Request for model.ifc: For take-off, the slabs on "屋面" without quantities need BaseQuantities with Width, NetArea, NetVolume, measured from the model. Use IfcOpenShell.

First a look at what the model holds.

```python
import ifcopenshell
import ifcopenshell.util.element
import ifcopenshell.util.unit

model = ifcopenshell.open("model.ifc")
print(model.schema)
for unit_type in ("LENGTHUNIT", "AREAUNIT", "VOLUMEUNIT"):
    print(unit_type, ifcopenshell.util.unit.calculate_unit_scale(model, unit_type))
storey = next(s for s in model.by_type("IfcBuildingStorey") if s.Name == "屋面")
slabs = [e for e in ifcopenshell.util.element.get_decomposition(storey) if e.is_a("IfcSlab")]
for e in sorted(slabs, key=lambda e: e.id()):
    print(e.id(), e.is_a(), e.Name, list(ifcopenshell.util.element.get_psets(e, qtos_only=True)), sep=" | ")
```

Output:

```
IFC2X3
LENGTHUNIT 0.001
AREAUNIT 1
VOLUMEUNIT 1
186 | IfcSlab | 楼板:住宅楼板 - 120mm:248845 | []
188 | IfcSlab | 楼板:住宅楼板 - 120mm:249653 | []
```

```python
import ifcopenshell
import ifcopenshell.api.pset
import ifcopenshell.geom
import ifcopenshell.util.element
import ifcopenshell.util.shape
import ifcopenshell.util.unit

model = ifcopenshell.open("model.ifc")
unit_scale = ifcopenshell.util.unit.calculate_unit_scale(model)
area_scale = ifcopenshell.util.unit.calculate_unit_scale(model, "AREAUNIT")
volume_scale = ifcopenshell.util.unit.calculate_unit_scale(model, "VOLUMEUNIT")
settings = ifcopenshell.geom.settings()

storey = next(s for s in model.by_type("IfcBuildingStorey") if s.Name == "屋面")
slabs = [e for e in ifcopenshell.util.element.get_decomposition(storey) if e.is_a("IfcSlab")]

for e in sorted(slabs, key=lambda e: e.id()):
    if ifcopenshell.util.element.get_psets(e, qtos_only=True, should_inherit=False):
        continue
    # Geometry comes back in metres, in the element's own axes.
    shape = ifcopenshell.geom.create_shape(settings, e)
    values = {
        "Width": ifcopenshell.util.shape.get_z(shape.geometry) / unit_scale,
        "NetArea": ifcopenshell.util.shape.get_footprint_area(shape.geometry) / area_scale,
        "NetVolume": ifcopenshell.util.shape.get_volume(shape.geometry) / volume_scale,
    }
    qto = ifcopenshell.api.pset.add_qto(model, product=e, name="BaseQuantities")
    ifcopenshell.api.pset.edit_qto(model, qto=qto, properties=values)
    print(e.id(), {k: round(v, 3) for k, v in values.items()})

model.write("model_v2.ifc")
```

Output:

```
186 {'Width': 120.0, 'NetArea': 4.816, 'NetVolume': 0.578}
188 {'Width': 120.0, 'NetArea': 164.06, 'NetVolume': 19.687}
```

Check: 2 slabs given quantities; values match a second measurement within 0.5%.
